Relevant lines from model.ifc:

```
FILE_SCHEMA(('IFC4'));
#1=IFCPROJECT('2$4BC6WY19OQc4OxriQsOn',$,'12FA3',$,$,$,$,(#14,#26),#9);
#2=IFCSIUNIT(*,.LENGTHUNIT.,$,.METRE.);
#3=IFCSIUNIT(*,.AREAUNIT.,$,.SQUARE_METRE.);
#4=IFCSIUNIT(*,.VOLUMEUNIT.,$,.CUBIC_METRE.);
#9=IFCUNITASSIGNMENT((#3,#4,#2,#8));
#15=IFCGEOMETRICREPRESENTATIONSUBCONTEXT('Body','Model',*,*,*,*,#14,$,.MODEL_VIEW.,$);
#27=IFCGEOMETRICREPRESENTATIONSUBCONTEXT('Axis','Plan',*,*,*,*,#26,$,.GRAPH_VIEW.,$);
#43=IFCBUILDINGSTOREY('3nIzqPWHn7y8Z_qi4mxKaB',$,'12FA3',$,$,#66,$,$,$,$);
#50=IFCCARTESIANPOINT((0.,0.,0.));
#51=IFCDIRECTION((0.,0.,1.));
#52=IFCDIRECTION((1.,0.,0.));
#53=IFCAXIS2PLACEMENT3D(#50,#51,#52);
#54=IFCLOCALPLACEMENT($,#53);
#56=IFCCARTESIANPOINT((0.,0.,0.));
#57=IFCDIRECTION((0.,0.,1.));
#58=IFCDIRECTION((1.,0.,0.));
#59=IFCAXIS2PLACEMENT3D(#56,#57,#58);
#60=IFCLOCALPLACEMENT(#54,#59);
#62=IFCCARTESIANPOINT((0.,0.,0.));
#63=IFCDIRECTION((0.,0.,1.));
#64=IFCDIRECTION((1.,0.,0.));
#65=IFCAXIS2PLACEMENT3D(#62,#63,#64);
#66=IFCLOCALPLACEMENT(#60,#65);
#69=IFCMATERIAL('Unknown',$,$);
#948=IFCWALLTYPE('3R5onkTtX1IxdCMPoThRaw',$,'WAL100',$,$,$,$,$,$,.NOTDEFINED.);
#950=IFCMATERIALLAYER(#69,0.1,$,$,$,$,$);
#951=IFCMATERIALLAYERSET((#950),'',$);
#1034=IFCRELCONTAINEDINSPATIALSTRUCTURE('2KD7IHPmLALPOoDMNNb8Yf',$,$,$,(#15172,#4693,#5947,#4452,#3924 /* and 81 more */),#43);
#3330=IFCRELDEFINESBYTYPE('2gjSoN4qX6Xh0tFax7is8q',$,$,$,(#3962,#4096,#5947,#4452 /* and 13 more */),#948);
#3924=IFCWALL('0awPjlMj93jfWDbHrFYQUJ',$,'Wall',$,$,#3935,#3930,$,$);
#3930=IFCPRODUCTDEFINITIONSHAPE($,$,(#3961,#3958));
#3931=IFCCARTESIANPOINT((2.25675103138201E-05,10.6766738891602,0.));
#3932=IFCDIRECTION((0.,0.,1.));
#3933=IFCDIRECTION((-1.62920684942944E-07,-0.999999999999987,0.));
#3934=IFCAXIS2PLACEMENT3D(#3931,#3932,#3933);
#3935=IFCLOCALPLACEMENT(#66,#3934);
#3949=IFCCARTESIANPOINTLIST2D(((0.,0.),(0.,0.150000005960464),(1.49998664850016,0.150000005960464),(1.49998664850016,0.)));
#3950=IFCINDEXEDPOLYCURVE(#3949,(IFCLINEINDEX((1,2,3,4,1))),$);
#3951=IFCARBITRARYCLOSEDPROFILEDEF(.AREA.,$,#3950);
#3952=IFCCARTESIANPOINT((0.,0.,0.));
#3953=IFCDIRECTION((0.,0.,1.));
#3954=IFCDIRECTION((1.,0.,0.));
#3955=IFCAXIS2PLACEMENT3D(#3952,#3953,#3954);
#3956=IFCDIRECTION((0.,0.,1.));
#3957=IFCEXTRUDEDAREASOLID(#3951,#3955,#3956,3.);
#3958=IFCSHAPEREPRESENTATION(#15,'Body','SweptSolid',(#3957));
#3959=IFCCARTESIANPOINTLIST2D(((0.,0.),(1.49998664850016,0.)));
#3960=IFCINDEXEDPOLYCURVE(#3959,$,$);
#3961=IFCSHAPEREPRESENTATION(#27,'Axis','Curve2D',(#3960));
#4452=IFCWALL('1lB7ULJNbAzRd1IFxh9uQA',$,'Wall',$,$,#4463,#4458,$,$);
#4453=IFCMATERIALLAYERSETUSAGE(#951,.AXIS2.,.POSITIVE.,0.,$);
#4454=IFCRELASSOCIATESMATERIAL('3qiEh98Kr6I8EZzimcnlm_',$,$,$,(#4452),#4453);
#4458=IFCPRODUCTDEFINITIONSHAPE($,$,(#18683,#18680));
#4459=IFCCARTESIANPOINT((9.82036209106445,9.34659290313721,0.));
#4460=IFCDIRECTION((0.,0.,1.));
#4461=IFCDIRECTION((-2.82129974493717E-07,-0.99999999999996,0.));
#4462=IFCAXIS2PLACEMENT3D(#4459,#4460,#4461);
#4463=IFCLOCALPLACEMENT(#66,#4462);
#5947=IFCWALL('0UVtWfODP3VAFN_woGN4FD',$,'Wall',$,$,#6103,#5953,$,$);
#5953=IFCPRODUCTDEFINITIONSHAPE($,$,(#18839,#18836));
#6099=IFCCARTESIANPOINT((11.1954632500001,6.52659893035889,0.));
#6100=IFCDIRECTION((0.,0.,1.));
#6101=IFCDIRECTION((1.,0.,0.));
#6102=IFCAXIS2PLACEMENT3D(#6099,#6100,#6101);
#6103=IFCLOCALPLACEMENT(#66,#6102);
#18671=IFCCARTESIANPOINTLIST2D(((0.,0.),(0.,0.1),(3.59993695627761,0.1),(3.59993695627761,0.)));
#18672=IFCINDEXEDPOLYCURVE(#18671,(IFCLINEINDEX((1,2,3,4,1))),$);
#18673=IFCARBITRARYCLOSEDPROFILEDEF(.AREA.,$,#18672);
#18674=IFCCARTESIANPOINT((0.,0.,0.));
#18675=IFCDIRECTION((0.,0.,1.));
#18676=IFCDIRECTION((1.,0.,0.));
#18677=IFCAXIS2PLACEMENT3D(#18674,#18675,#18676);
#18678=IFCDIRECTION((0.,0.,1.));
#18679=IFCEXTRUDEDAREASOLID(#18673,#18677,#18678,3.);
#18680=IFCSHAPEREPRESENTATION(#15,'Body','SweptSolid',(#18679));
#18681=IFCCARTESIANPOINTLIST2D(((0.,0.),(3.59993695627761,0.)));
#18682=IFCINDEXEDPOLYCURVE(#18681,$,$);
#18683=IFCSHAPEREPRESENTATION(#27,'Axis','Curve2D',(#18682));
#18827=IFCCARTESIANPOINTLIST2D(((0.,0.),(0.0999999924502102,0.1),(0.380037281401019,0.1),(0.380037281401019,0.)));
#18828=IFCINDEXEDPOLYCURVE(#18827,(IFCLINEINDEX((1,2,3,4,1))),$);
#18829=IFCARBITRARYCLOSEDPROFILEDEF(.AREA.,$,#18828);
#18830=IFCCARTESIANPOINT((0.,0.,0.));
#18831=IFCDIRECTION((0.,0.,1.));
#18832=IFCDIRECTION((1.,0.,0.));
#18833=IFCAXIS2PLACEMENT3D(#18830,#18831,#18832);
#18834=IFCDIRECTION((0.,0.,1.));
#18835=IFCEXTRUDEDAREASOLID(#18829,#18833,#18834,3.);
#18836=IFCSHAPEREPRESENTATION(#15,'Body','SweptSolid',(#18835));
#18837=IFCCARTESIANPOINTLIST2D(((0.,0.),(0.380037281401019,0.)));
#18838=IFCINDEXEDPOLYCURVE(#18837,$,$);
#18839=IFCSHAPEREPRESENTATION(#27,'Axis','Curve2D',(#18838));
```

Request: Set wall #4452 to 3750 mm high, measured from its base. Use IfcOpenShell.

```python
import ifcopenshell
import ifcopenshell.geom
import ifcopenshell.util.representation
import ifcopenshell.util.shape
import ifcopenshell.util.unit

model = ifcopenshell.open("model.ifc")
unit_scale = ifcopenshell.util.unit.calculate_unit_scale(model)
settings = ifcopenshell.geom.settings()


def volume(element):
    """Net volume in cubic metres, openings subtracted."""
    shape = ifcopenshell.geom.create_shape(settings, element)
    return ifcopenshell.util.shape.get_volume(shape.geometry)


wall = model.by_id(4452)
before = volume(wall)

body = ifcopenshell.util.representation.get_representation(wall, "Model", "Body")
solid = body.Items[0]
old_height = solid.Depth
solid.Depth = 3.75 / unit_scale
after = volume(wall)

print(f"height {old_height:g} -> {solid.Depth:g}, volume {before:.3f} -> {after:.3f} m3")

model.write("model_edited.ifc")
```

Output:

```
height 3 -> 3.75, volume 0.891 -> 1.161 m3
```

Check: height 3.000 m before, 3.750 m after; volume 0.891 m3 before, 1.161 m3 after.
